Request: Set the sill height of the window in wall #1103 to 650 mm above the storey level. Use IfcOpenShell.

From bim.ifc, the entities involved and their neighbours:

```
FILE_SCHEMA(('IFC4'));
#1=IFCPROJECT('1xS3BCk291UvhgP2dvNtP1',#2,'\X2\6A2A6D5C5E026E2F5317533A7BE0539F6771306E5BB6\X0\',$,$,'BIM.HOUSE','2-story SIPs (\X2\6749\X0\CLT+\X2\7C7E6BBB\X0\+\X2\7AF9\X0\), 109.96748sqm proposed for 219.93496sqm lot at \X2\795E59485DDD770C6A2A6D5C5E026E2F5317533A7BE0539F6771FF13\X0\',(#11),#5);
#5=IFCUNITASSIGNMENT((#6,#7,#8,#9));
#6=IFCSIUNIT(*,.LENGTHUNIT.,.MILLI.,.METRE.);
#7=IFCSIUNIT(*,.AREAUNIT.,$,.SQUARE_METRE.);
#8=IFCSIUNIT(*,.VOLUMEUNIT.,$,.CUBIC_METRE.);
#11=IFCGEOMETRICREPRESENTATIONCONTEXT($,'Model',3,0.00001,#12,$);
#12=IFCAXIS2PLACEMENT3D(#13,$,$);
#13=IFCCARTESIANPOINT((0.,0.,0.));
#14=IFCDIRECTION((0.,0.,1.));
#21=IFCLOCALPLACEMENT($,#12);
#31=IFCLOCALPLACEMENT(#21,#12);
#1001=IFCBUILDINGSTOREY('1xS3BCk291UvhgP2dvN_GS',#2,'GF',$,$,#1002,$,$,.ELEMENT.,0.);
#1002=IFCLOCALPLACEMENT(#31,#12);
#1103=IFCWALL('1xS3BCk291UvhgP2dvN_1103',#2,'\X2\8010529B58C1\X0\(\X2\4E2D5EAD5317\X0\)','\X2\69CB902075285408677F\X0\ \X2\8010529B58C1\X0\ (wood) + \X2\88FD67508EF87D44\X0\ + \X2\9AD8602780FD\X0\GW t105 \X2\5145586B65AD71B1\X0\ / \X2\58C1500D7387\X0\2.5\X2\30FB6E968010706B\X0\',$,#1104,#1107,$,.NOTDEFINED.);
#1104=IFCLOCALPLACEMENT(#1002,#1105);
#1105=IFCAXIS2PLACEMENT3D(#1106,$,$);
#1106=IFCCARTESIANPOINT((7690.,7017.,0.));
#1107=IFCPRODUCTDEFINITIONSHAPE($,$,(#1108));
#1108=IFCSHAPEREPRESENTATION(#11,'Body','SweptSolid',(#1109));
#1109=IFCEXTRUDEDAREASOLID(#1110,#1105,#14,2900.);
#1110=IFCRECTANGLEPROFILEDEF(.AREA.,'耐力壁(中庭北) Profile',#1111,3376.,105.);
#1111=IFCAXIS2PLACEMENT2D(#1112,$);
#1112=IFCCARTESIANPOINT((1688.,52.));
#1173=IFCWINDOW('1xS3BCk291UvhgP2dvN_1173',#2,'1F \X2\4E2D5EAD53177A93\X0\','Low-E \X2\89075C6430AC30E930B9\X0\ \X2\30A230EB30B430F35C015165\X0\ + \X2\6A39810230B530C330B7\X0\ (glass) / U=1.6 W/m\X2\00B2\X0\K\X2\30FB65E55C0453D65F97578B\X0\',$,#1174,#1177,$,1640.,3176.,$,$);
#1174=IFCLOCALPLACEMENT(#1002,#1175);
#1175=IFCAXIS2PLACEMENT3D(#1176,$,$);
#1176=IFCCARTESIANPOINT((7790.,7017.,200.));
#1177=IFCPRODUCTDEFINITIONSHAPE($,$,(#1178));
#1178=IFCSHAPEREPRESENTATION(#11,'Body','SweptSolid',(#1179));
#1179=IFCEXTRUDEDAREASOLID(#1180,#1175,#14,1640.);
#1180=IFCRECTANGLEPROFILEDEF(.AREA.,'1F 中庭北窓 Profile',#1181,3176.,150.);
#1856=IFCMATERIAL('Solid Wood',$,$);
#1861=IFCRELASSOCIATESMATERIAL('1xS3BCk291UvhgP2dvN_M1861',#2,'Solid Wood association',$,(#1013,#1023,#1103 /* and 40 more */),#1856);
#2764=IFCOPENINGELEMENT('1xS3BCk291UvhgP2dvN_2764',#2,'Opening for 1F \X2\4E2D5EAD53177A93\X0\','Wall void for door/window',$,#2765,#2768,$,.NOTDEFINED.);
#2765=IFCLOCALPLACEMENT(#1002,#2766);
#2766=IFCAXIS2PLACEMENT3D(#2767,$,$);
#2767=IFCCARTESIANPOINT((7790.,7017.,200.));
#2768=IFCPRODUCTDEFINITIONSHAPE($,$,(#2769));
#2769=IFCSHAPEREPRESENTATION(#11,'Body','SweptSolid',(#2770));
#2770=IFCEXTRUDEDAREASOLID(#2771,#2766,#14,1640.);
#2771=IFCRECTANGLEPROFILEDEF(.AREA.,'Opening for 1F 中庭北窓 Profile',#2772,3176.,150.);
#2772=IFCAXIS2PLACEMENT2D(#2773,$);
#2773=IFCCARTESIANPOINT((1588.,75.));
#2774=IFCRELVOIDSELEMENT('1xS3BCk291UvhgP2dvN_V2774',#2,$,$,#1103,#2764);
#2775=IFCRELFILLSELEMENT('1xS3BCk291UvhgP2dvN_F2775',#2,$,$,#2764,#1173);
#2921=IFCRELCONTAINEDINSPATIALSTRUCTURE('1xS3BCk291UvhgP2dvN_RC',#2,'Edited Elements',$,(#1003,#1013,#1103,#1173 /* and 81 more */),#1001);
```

```python
import numpy as np
import ifcopenshell
import ifcopenshell.api.geometry
import ifcopenshell.geom
import ifcopenshell.util.element
import ifcopenshell.util.placement
import ifcopenshell.util.shape
import ifcopenshell.util.unit

model = ifcopenshell.open("bim.ifc")
unit_scale = ifcopenshell.util.unit.calculate_unit_scale(model)

window = model.by_id(1173)
opening = window.FillsVoids[0].RelatingOpeningElement
storey = ifcopenshell.util.element.get_container(window, ifc_class="IfcBuildingStorey")
level = ifcopenshell.util.placement.get_local_placement(storey.ObjectPlacement)[2, 3]

# The opening's origin need not be at the sill, so measure its lowest point.
shape = ifcopenshell.geom.create_shape(ifcopenshell.geom.settings(), opening)
bottom = ifcopenshell.util.shape.get_shape_bottom_elevation(shape, shape.geometry) / unit_scale
dz = level + 0.65 / unit_scale - bottom

shift = np.array([0.0, 0.0, dz])
# The window is not placed relative to its opening, so move both.
for product in (opening, window):
    matrix = ifcopenshell.util.placement.get_local_placement(product.ObjectPlacement)
    matrix[:3, 3] += shift
    ifcopenshell.api.geometry.edit_object_placement(model, product=product, matrix=matrix, is_si=False)

print(f"moved by {dz * unit_scale:+.3f} m")

model.write("bim-out.ifc")
```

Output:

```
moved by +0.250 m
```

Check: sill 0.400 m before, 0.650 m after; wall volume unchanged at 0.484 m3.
